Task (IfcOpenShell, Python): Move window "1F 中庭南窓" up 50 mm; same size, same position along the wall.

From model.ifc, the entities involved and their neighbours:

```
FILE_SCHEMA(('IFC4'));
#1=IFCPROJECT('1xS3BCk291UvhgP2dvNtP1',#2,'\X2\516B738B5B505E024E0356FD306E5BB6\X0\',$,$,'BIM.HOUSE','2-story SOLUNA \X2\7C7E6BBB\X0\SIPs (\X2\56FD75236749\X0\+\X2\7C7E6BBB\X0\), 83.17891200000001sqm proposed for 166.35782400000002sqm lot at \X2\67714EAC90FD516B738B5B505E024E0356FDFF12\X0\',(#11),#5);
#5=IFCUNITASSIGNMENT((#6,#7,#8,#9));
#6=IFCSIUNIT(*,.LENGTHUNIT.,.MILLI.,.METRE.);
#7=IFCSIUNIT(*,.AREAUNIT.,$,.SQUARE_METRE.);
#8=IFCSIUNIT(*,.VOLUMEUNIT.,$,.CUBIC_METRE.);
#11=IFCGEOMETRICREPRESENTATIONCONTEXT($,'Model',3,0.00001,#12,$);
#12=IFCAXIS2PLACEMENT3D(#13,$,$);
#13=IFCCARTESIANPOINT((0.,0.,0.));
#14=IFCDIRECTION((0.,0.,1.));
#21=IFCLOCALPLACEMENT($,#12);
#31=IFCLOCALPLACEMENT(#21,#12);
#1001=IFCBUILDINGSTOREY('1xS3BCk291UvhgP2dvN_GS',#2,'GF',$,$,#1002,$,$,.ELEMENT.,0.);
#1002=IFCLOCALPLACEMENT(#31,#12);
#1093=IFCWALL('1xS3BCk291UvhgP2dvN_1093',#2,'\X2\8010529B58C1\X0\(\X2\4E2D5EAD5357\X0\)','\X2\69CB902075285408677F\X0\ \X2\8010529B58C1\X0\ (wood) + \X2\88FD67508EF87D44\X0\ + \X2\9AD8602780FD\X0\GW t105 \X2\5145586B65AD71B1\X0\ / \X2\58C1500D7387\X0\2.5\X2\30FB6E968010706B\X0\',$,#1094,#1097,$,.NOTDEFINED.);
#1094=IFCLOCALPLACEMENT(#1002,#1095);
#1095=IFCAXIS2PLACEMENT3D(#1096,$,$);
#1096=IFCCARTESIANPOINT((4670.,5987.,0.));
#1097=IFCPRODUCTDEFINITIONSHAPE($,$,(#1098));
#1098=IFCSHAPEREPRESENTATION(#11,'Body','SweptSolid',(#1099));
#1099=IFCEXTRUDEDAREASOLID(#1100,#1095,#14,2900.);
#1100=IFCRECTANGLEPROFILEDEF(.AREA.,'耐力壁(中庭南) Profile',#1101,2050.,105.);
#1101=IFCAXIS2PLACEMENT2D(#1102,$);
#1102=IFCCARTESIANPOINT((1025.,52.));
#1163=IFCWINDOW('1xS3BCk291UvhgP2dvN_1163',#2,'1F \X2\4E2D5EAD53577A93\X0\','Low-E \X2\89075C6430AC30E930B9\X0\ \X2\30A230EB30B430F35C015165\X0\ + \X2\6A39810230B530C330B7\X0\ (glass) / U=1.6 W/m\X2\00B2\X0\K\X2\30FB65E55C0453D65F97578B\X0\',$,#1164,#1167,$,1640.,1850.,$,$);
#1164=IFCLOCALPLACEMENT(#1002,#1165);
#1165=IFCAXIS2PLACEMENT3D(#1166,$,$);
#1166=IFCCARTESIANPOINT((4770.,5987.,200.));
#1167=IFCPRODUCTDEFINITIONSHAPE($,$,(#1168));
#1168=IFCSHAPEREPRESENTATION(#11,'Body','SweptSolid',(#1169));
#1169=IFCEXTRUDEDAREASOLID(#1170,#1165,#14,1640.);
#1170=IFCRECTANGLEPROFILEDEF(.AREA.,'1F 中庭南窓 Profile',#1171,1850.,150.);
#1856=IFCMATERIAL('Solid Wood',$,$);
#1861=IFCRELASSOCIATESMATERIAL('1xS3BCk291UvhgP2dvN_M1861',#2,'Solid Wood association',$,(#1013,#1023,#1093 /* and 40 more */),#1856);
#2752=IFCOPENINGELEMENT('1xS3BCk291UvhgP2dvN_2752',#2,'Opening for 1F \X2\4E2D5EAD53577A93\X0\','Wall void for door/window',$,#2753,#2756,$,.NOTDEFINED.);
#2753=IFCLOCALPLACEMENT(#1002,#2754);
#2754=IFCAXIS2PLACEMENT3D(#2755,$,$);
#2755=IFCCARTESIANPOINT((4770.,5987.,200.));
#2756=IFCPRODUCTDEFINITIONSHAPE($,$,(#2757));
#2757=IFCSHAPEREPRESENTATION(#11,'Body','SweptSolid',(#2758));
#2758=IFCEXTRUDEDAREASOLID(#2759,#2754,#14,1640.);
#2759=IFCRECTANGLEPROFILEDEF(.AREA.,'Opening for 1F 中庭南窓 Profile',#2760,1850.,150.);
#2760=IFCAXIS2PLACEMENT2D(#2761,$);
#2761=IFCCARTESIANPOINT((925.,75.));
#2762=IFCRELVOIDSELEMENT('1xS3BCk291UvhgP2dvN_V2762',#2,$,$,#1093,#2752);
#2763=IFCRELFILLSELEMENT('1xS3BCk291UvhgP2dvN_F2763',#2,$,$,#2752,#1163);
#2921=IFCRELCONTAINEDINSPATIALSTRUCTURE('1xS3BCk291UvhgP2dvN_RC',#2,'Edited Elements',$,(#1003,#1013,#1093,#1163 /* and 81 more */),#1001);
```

```python
import numpy as np
import ifcopenshell
import ifcopenshell.api.geometry
import ifcopenshell.util.placement
import ifcopenshell.util.unit

model = ifcopenshell.open("model.ifc")
unit_scale = ifcopenshell.util.unit.calculate_unit_scale(model)

window = model.by_id(1163)
opening = window.FillsVoids[0].RelatingOpeningElement
dz = 0.05 / unit_scale

shift = np.array([0.0, 0.0, dz])
# The window is not placed relative to its opening, so move both.
for product in (opening, window):
    matrix = ifcopenshell.util.placement.get_local_placement(product.ObjectPlacement)
    matrix[:3, 3] += shift
    ifcopenshell.api.geometry.edit_object_placement(model, product=product, matrix=matrix, is_si=False)

print(f"moved by {dz * unit_scale:+.3f} m")

model.write("model_rev.ifc")
```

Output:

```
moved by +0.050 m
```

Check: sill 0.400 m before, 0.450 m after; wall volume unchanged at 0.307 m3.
